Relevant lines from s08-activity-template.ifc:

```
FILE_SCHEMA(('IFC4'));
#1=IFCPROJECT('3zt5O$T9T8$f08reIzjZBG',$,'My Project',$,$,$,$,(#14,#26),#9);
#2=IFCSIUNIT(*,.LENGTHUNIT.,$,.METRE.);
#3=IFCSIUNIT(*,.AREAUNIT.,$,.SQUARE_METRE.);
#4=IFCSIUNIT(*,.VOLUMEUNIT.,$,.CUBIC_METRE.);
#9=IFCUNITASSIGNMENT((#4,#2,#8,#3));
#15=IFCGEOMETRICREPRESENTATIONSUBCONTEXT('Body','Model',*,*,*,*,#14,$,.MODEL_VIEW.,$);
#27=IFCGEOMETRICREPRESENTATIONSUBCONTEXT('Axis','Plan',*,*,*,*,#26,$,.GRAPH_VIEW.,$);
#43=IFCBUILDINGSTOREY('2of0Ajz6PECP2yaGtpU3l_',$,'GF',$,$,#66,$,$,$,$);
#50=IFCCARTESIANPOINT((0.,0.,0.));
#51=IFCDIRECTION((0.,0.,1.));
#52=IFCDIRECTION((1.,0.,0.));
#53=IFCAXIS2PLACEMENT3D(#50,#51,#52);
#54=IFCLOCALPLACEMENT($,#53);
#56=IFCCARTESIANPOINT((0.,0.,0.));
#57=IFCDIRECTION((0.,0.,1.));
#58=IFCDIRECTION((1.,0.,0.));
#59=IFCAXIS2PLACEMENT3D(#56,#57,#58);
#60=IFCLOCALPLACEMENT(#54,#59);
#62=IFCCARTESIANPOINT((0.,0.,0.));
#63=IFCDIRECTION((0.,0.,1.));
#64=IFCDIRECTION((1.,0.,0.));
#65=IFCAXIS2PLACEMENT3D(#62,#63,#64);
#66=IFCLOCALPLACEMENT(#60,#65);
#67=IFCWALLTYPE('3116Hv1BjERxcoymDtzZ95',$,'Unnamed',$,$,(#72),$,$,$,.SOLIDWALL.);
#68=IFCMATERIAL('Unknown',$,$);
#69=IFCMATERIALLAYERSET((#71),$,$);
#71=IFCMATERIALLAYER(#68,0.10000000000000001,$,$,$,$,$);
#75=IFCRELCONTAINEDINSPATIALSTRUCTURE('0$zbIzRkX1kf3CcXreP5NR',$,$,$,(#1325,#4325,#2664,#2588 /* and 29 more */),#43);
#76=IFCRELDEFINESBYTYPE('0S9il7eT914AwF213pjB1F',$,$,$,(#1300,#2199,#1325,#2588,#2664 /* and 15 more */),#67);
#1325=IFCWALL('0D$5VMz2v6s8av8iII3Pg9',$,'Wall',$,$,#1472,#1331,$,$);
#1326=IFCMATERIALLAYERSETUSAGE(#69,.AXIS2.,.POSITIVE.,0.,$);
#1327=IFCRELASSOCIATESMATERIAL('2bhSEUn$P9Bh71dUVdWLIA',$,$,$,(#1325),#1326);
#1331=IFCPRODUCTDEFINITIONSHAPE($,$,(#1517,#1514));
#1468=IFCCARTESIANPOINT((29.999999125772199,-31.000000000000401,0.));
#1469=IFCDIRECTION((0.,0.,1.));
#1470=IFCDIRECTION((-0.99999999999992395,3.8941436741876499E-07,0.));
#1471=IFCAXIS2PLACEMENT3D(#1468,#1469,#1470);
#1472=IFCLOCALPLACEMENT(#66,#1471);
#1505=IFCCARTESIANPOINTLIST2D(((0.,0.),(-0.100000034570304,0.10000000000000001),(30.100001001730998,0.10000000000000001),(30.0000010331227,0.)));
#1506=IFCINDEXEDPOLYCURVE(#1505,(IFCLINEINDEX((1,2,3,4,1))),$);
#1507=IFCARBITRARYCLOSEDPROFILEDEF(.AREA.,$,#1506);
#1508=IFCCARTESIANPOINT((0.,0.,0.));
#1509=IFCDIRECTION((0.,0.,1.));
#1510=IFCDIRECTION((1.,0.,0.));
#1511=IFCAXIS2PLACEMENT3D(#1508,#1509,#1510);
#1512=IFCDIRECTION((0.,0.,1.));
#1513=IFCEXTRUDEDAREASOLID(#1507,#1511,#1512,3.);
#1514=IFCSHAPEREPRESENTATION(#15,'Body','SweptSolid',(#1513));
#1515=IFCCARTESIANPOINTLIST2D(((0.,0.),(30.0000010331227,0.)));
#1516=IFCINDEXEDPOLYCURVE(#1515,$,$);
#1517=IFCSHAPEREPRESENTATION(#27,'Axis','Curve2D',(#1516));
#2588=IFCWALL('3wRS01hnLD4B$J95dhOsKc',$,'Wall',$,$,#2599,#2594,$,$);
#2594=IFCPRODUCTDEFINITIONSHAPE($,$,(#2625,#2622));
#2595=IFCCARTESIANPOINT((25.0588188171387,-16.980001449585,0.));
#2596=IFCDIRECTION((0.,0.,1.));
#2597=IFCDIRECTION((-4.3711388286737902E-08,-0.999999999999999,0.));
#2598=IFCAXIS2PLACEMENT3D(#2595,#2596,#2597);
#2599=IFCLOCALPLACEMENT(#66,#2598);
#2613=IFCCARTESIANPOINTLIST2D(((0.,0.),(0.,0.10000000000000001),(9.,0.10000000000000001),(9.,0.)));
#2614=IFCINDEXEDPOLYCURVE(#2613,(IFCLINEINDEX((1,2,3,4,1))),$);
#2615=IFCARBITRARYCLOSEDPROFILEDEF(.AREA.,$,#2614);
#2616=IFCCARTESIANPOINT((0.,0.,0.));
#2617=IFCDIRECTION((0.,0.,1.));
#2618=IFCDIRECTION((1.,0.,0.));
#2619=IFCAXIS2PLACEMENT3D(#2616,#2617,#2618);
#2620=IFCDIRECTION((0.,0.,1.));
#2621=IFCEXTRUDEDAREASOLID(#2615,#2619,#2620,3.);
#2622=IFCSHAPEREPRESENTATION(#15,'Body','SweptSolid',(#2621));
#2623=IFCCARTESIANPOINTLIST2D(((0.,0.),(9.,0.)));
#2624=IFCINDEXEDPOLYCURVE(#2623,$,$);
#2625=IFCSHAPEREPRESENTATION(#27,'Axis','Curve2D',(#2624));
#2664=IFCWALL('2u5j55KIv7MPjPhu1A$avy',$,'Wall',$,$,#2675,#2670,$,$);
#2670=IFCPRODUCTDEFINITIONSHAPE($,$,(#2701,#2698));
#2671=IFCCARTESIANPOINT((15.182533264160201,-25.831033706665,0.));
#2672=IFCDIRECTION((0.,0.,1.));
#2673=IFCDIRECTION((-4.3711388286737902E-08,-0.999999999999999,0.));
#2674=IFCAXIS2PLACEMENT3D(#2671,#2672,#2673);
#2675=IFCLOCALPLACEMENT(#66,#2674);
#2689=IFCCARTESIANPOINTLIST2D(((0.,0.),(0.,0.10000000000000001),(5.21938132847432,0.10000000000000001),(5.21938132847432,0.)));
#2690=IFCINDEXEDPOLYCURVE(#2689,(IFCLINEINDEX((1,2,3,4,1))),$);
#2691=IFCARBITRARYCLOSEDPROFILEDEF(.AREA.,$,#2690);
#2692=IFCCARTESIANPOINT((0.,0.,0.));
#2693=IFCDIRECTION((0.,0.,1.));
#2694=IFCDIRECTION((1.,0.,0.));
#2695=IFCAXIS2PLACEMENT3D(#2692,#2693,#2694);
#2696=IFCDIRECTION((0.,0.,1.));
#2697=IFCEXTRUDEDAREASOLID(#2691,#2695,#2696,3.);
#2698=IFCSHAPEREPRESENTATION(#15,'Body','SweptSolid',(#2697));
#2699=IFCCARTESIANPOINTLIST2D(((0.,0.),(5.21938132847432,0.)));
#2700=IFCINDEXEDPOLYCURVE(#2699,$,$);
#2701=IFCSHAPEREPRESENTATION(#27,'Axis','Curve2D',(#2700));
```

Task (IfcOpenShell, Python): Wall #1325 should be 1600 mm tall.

```python
import ifcopenshell
import ifcopenshell.geom
import ifcopenshell.util.representation
import ifcopenshell.util.shape

model = ifcopenshell.open("s08-activity-template.ifc")
settings = ifcopenshell.geom.settings()


def volume(element):
    """Net volume in cubic metres, openings subtracted."""
    shape = ifcopenshell.geom.create_shape(settings, element)
    return ifcopenshell.util.shape.get_volume(shape.geometry)


wall = model.by_guid("0D$5VMz2v6s8av8iII3Pg9")
before = volume(wall)

body = ifcopenshell.util.representation.get_representation(wall, "Model", "Body")
solid = body.Items[0]
old_height = solid.Depth
solid.Depth = 1.6
after = volume(wall)

print(f"height {old_height:g} -> {solid.Depth:g}, volume {before:.3f} -> {after:.3f} m3")

model.write("s08-activity-template_rev.ifc")
```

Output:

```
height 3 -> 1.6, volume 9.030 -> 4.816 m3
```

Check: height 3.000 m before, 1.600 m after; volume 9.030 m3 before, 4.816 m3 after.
